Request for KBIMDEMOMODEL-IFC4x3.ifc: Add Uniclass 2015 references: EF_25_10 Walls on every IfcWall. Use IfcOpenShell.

First a look at what the model holds.

```python
import ifcopenshell

model = ifcopenshell.open("KBIMDEMOMODEL-IFC4x3.ifc")
print(model.schema)
print("classifications:", [c.Name for c in model.by_type("IfcClassification")])
for ifc_class in ("IfcDoor", "IfcRoof", "IfcStair", "IfcWall", "IfcWindow"):
    print(ifc_class, len(model.by_type(ifc_class)))
```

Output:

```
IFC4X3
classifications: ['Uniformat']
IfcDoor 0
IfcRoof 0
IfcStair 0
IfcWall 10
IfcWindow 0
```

```python
import ifcopenshell
import ifcopenshell.api.classification

model = ifcopenshell.open("KBIMDEMOMODEL-IFC4x3.ifc")

system = ifcopenshell.api.classification.add_classification(model, classification="Uniclass 2015")

codes = {
    "IfcWall": ("EF_25_10", "Walls"),
}
for ifc_class, (code, name) in codes.items():
    products = model.by_type(ifc_class)
    ifcopenshell.api.classification.add_reference(
        model, products=products, classification=system, identification=code, name=name
    )
    print(code, len(products))

model.write("KBIMDEMOMODEL-IFC4x3_rev.ifc")
```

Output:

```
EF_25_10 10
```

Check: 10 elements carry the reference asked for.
